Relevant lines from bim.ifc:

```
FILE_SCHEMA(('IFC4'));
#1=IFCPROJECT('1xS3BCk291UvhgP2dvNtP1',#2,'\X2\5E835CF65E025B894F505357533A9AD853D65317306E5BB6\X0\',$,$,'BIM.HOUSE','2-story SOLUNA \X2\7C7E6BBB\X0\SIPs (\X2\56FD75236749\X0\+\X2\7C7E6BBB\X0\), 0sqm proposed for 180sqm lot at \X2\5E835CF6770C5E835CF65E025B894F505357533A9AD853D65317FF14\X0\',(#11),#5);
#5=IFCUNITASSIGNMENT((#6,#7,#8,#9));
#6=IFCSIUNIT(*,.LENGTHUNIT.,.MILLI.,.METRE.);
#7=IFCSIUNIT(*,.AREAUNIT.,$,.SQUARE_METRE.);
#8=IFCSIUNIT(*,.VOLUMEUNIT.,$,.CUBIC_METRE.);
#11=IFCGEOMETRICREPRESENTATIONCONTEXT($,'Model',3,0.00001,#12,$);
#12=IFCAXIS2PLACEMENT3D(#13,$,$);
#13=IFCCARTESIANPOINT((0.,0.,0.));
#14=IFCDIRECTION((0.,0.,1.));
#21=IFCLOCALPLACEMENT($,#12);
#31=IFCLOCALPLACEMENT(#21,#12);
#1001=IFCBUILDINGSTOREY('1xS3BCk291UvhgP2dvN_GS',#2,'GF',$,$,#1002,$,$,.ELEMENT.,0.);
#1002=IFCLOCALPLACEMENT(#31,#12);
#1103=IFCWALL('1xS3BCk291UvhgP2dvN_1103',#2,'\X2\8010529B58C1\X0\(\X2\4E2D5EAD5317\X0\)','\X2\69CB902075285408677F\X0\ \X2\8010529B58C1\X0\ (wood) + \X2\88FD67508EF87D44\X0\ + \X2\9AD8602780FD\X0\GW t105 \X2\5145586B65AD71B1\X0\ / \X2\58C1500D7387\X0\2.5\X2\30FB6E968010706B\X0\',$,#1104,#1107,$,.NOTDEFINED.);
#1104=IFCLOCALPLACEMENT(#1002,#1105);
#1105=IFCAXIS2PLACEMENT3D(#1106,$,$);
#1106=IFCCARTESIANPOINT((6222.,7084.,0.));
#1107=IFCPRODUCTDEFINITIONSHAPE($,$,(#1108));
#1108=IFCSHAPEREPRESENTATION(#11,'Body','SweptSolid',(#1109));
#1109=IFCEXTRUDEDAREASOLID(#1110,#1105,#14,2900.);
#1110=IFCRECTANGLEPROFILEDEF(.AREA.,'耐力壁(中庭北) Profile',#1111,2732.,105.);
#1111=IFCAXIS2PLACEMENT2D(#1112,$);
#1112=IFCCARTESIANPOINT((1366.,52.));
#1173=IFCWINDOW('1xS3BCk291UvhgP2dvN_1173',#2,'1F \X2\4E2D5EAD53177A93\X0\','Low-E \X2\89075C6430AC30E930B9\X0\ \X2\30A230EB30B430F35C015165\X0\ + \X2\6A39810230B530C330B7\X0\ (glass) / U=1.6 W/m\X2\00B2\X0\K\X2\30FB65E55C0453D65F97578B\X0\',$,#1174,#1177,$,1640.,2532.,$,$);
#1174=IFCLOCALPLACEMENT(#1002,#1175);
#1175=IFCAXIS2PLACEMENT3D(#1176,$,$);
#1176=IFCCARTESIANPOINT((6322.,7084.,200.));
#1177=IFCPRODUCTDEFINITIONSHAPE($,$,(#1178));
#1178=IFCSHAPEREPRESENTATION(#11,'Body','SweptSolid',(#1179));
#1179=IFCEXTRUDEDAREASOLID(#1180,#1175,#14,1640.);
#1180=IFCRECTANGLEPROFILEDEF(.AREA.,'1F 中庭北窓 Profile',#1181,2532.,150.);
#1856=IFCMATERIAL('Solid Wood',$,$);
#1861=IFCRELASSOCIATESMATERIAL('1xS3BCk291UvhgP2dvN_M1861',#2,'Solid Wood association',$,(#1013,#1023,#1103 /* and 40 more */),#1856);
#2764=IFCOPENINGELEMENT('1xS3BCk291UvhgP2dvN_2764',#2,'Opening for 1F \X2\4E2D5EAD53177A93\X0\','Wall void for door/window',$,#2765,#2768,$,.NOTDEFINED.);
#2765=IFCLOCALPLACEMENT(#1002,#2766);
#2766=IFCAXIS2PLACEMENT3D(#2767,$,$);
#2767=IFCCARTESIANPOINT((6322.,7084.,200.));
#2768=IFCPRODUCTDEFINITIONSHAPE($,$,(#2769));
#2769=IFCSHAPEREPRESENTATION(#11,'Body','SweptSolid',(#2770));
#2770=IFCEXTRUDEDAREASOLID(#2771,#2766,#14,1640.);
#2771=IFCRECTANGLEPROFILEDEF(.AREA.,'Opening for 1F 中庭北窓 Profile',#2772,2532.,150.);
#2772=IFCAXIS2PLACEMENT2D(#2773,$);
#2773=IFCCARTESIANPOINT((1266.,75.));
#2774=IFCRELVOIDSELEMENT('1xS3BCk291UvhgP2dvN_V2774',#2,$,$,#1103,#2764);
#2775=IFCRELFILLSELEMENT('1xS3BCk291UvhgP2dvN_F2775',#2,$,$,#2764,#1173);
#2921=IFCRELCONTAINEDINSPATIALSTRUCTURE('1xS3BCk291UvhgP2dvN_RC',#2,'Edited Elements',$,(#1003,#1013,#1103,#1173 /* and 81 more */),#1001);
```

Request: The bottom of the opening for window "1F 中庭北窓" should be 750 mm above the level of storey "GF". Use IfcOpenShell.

```python
import numpy as np
import ifcopenshell
import ifcopenshell.api.geometry
import ifcopenshell.geom
import ifcopenshell.util.element
import ifcopenshell.util.placement
import ifcopenshell.util.shape
import ifcopenshell.util.unit

model = ifcopenshell.open("bim.ifc")
unit_scale = ifcopenshell.util.unit.calculate_unit_scale(model)

window = model.by_guid("1xS3BCk291UvhgP2dvN_1173")
opening = window.FillsVoids[0].RelatingOpeningElement
storey = ifcopenshell.util.element.get_container(window, ifc_class="IfcBuildingStorey")
level = ifcopenshell.util.placement.get_local_placement(storey.ObjectPlacement)[2, 3]

# The opening's origin need not be at the sill, so measure its lowest point.
shape = ifcopenshell.geom.create_shape(ifcopenshell.geom.settings(), opening)
bottom = ifcopenshell.util.shape.get_shape_bottom_elevation(shape, shape.geometry) / unit_scale
dz = level + 0.75 / unit_scale - bottom

shift = np.array([0.0, 0.0, dz])
# The window is not placed relative to its opening, so move both.
for product in (opening, window):
    matrix = ifcopenshell.util.placement.get_local_placement(product.ObjectPlacement)
    matrix[:3, 3] += shift
    ifcopenshell.api.geometry.edit_object_placement(model, product=product, matrix=matrix, is_si=False)

print(f"moved by {dz * unit_scale:+.3f} m")

model.write("bim-out.ifc")
```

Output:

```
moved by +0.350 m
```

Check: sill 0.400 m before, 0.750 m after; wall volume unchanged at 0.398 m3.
